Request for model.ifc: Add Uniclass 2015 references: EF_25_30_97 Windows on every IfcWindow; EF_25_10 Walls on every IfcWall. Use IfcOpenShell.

First a look at what the model holds.

```python
import ifcopenshell

model = ifcopenshell.open("model.ifc")
print(model.schema)
print("classifications:", [c.Name for c in model.by_type("IfcClassification")])
for ifc_class in ("IfcDoor", "IfcRoof", "IfcStair", "IfcWall", "IfcWindow"):
    print(ifc_class, len(model.by_type(ifc_class)))
```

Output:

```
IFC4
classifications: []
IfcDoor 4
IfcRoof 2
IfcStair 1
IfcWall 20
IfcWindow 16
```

```python
import ifcopenshell
import ifcopenshell.api.classification

model = ifcopenshell.open("model.ifc")

system = ifcopenshell.api.classification.add_classification(model, classification="Uniclass 2015")

codes = {
    "IfcWindow": ("EF_25_30_97", "Windows"),
    "IfcWall": ("EF_25_10", "Walls"),
}
for ifc_class, (code, name) in codes.items():
    products = model.by_type(ifc_class)
    ifcopenshell.api.classification.add_reference(
        model, products=products, classification=system, identification=code, name=name
    )
    print(code, len(products))

model.write("model_rev.ifc")
```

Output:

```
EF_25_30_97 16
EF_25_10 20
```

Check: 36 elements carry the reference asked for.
